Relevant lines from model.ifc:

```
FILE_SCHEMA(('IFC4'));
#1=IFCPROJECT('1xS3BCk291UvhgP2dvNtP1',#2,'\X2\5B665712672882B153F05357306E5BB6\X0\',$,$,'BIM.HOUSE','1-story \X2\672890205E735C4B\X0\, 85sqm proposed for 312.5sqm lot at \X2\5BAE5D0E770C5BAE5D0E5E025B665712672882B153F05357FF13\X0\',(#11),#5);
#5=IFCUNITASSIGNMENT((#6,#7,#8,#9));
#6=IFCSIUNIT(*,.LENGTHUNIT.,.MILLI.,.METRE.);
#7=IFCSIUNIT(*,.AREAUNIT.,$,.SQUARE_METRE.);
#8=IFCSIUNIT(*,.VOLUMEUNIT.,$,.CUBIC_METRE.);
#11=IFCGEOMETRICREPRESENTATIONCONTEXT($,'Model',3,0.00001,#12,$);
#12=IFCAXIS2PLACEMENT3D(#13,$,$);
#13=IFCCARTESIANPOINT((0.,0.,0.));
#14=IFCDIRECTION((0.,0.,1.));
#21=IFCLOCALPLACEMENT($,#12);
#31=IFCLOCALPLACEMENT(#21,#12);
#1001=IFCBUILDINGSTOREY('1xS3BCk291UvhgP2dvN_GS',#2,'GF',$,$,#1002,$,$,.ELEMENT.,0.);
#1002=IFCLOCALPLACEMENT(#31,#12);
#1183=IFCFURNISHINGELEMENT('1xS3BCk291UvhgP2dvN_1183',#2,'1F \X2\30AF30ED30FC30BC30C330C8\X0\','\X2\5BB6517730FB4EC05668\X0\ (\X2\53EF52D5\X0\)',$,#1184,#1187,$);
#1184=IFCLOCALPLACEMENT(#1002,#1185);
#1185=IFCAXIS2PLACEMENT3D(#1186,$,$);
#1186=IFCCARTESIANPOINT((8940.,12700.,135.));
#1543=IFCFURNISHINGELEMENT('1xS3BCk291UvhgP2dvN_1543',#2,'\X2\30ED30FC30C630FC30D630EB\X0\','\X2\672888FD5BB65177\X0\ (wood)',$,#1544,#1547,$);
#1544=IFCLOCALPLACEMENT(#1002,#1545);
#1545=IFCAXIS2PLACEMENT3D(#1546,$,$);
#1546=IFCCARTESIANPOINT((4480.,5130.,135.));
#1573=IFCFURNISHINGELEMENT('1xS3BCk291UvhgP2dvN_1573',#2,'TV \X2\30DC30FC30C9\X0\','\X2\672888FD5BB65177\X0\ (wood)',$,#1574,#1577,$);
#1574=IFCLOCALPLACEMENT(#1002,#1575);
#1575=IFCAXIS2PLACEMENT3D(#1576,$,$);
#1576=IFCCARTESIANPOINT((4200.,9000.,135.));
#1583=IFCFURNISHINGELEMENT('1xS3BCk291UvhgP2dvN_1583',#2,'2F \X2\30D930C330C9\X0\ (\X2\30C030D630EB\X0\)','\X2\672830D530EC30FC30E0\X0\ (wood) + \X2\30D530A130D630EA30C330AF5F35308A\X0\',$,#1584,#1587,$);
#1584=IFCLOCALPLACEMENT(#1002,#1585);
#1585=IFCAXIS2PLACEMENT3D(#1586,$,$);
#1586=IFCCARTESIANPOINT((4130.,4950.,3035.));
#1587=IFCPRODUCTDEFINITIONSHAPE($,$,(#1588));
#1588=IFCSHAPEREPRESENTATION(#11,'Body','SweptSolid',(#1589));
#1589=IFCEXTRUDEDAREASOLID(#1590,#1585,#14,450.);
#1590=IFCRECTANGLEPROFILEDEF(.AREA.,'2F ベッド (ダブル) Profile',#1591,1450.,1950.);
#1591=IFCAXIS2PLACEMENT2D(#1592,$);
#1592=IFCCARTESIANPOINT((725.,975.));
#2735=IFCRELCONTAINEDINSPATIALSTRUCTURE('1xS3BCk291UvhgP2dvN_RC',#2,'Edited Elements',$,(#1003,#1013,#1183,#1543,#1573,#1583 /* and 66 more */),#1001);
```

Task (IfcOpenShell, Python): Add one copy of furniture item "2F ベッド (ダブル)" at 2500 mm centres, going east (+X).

```python
import numpy as np
import ifcopenshell
import ifcopenshell.api.geometry
import ifcopenshell.api.root
import ifcopenshell.util.element
import ifcopenshell.util.placement

model = ifcopenshell.open("model.ifc")


def reuse_history(source, copy):
    """copy_class also copies each property set's owner history, people and application; keep the originals."""
    for rel in copy.IsDefinedBy:
        if rel.is_a("IfcRelDefinesByProperties") and (history := rel.RelatingPropertyDefinition.OwnerHistory):
            rel.RelatingPropertyDefinition.OwnerHistory = source.OwnerHistory
            ifcopenshell.util.element.remove_deep2(model, history)


source = model.by_guid("1xS3BCk291UvhgP2dvN_1583")
base = ifcopenshell.util.placement.get_local_placement(source.ObjectPlacement)
step = np.array([1.0, 0.0, 0.0]) * 2500.0

for i in range(1, 2):
    copy = ifcopenshell.api.root.copy_class(model, product=source)
    copy.Representation = ifcopenshell.util.element.copy_deep(
        model, source.Representation, exclude=["IfcGeometricRepresentationContext", "IfcRepresentationMap"]
    )
    reuse_history(source, copy)
    matrix = base.copy()
    matrix[:3, 3] += i * step
    print("added at", matrix[:3, 3].round(3) + 0.0)
    ifcopenshell.api.geometry.edit_object_placement(model, product=copy, matrix=matrix, is_si=False)

model.write("model-out.ifc")
```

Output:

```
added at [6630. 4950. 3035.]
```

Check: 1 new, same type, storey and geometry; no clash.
